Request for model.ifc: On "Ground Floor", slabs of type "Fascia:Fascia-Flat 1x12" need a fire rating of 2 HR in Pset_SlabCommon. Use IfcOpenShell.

First a look at what the model holds.

```python
import ifcopenshell
import ifcopenshell.util.element

model = ifcopenshell.open("model.ifc")
print(model.schema)
storey = next(s for s in model.by_type("IfcBuildingStorey") if s.Name == "Ground Floor")
slabs = [e for e in ifcopenshell.util.element.get_decomposition(storey) if e.is_a("IfcSlab")]
seen = {}
for e in slabs:
    element_type = ifcopenshell.util.element.get_type(e)
    key = (element_type.Name if element_type != e and element_type else None, ifcopenshell.util.element.get_pset(e, "Pset_SlabCommon", "FireRating"))
    seen[key] = seen.get(key, 0) + 1
for (name, value), count in sorted(seen.items(), key=str):
    print(count, "x", name, "|", value)
```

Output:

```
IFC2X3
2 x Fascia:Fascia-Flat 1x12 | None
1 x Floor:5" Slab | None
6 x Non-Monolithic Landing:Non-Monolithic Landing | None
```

```python
import ifcopenshell
import ifcopenshell.api.pset
import ifcopenshell.util.element

model = ifcopenshell.open("model.ifc")

storey = next(s for s in model.by_type("IfcBuildingStorey") if s.Name == "Ground Floor")
slabs = [e for e in ifcopenshell.util.element.get_decomposition(storey) if e.is_a("IfcSlab")]

count = 0
for e in slabs:
    element_type = ifcopenshell.util.element.get_type(e)
    if element_type in (None, e) or element_type.Name != "Fascia:Fascia-Flat 1x12":
        continue
    # add_pset returns the element's existing set when there is one.
    pset = ifcopenshell.api.pset.add_pset(model, product=e, name="Pset_SlabCommon")
    ifcopenshell.api.pset.edit_pset(model, pset=pset, properties={"FireRating": "2 HR"})
    count += 1

print(count, "slabs updated")

model.write("model-out.ifc")
```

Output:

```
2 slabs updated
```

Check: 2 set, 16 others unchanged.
